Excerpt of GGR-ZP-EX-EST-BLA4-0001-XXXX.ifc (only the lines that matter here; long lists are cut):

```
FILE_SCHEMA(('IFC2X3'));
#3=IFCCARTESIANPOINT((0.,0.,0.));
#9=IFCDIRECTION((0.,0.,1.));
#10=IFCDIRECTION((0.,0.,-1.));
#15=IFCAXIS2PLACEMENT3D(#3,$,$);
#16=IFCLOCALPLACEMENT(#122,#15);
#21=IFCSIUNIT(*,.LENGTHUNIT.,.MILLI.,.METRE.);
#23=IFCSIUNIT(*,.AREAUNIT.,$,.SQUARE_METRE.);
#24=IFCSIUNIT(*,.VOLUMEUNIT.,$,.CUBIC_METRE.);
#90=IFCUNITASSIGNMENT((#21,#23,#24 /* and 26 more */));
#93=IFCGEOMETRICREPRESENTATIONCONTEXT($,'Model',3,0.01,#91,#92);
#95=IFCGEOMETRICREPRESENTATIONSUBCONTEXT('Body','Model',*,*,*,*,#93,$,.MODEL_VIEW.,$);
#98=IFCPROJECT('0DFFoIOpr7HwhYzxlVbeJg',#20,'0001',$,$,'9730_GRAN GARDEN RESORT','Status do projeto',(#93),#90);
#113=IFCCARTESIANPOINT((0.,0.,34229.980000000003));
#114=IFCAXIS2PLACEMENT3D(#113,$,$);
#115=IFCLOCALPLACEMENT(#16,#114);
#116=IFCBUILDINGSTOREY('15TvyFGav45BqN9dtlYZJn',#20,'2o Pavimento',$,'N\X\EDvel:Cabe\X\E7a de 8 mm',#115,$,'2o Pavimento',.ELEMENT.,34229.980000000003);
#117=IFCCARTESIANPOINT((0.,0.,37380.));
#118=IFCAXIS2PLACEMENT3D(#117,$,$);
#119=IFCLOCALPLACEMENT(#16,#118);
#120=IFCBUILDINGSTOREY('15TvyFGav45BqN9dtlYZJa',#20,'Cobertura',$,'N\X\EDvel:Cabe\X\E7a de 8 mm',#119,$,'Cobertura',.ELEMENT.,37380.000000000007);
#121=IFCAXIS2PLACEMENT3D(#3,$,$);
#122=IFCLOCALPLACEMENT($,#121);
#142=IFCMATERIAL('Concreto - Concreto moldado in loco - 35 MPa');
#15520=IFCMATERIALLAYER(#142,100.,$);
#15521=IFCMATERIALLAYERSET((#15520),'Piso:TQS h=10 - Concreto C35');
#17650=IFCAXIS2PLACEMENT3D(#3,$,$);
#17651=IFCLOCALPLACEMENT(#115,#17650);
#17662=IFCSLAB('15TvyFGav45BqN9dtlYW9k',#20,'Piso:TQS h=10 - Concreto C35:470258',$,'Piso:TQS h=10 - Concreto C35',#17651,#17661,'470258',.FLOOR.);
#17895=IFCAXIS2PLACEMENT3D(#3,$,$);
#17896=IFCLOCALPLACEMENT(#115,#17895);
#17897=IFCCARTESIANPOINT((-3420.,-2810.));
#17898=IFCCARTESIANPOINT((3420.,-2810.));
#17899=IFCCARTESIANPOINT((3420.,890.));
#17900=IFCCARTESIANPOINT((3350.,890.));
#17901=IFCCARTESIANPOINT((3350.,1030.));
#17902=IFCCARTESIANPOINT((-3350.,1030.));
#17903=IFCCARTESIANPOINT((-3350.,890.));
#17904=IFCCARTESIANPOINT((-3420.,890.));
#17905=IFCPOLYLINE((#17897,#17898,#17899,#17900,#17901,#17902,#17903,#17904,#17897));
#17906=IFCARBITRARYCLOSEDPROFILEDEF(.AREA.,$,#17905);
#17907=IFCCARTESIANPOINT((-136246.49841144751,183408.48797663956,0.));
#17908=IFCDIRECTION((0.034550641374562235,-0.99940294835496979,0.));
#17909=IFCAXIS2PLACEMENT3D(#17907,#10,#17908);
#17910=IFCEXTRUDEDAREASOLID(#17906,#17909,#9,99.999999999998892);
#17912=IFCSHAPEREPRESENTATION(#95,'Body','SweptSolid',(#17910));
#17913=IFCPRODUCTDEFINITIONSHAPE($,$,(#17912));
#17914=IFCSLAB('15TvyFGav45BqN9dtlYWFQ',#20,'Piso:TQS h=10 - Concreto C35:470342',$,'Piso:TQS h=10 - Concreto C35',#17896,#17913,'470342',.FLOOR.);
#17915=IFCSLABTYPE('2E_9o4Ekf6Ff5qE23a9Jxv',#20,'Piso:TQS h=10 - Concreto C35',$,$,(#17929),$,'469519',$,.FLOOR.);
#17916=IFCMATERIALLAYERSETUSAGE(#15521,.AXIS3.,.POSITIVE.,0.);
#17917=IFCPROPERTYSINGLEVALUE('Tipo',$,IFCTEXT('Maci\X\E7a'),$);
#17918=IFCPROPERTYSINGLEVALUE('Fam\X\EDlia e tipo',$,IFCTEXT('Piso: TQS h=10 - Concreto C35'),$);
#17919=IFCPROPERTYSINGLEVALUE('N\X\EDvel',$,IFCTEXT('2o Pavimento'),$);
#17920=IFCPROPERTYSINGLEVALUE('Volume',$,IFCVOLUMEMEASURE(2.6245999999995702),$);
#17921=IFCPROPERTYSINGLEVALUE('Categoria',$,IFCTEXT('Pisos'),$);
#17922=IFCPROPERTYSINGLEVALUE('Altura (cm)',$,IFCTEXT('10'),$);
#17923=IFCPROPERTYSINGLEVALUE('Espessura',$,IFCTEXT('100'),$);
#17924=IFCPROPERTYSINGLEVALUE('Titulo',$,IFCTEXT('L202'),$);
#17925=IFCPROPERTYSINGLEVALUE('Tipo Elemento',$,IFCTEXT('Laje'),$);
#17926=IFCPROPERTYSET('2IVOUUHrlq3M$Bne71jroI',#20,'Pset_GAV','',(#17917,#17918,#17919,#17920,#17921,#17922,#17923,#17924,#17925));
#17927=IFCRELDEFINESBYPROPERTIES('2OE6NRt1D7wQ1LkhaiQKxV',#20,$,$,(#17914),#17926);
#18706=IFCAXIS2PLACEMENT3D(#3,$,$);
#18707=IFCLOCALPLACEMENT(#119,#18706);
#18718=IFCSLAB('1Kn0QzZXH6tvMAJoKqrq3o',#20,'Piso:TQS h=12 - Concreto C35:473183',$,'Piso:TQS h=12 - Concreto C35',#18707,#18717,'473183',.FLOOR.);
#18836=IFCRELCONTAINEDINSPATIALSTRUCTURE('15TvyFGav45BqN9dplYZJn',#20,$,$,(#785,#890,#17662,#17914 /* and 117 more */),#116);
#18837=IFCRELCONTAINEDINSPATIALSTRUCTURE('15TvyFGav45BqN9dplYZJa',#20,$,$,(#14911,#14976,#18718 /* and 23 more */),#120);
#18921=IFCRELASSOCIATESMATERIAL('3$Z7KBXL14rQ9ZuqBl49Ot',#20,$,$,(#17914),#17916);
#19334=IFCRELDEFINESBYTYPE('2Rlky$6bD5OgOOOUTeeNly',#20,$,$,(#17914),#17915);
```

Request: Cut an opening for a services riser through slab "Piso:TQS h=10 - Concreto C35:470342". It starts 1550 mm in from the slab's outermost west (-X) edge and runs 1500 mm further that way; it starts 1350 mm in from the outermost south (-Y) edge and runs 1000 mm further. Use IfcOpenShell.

```python
import numpy as np
import ifcopenshell
import ifcopenshell.api.feature
import ifcopenshell.api.geometry
import ifcopenshell.api.pset
import ifcopenshell.api.root
import ifcopenshell.geom
import ifcopenshell.util.element
import ifcopenshell.util.placement
import ifcopenshell.util.representation
import ifcopenshell.util.shape
import ifcopenshell.util.unit

model = ifcopenshell.open("GGR-ZP-EX-EST-BLA4-0001-XXXX.ifc")
unit_scale = ifcopenshell.util.unit.calculate_unit_scale(model)
volume_scale = ifcopenshell.util.unit.calculate_unit_scale(model, "VOLUMEUNIT")
settings = ifcopenshell.geom.settings()


def volume(element):
    """Net volume in cubic metres, openings subtracted."""
    shape = ifcopenshell.geom.create_shape(settings, element)
    return ifcopenshell.util.shape.get_volume(shape.geometry)


slab = model.by_guid("15TvyFGav45BqN9dtlYWFQ")
before = volume(slab)

# Extent in the slab's own axes, in metres. The edges named are its -X and -Y sides.
slab_shape = ifcopenshell.geom.create_shape(settings, slab)
vertices = ifcopenshell.util.shape.get_vertices(slab_shape.geometry)
x_min, y_min, bottom = vertices.min(axis=0)
top = vertices[:, 2].max()

opening = ifcopenshell.api.root.create_entity(model, ifc_class="IfcOpeningElement", name="Services riser opening")
context = ifcopenshell.util.representation.get_context(model, "Model", "Body", "MODEL_VIEW")
width, depth = 1.5, 1
outline = [(0.0, 0.0), (width, 0.0), (width, depth), (0.0, depth), (0.0, 0.0)]
# Overshoot both faces by 50 mm so the cut is clean.
shape = ifcopenshell.api.geometry.add_slab_representation(
    model, context=context, depth=top - bottom + 0.1, polyline=outline
)
ifcopenshell.api.geometry.assign_representation(model, product=opening, representation=shape)

matrix = ifcopenshell.util.placement.get_local_placement(slab.ObjectPlacement)
matrix[:, 3] = matrix @ np.append(np.array([x_min + 1.55, y_min + 1.35, bottom - 0.05]) / unit_scale, 1.0)
ifcopenshell.api.geometry.edit_object_placement(model, product=opening, matrix=matrix, is_si=False)
ifcopenshell.api.feature.add_feature(model, feature=opening, element=slab)

after = volume(slab)

# Update the slab's stored quantities.
pset = model.by_id(ifcopenshell.util.element.get_pset(slab, "Pset_GAV", should_inherit=False)["id"])
ifcopenshell.api.pset.edit_pset(model, pset=pset, properties={
    "Volume": model.create_entity("IfcVolumeMeasure", after / volume_scale),
})

print(f"slab volume {before:.3f} -> {after:.3f} m3")

model.write("GGR-ZP-EX-EST-BLA4-0001-XXXX_edited.ifc")
```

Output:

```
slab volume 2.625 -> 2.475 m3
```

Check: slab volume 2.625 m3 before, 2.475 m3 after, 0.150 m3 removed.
